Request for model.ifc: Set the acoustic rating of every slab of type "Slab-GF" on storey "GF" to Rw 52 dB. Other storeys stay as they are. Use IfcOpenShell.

First a look at what the model holds.

```python
import ifcopenshell
import ifcopenshell.util.element

model = ifcopenshell.open("model.ifc")
print(model.schema)
storey = next(s for s in model.by_type("IfcBuildingStorey") if s.Name == "GF")
slabs = [e for e in ifcopenshell.util.element.get_decomposition(storey) if e.is_a("IfcSlab")]
seen = {}
for e in slabs:
    element_type = ifcopenshell.util.element.get_type(e)
    key = (element_type.Name if element_type != e and element_type else None, ifcopenshell.util.element.get_pset(e, "Pset_SlabCommon", "AcousticRating"))
    seen[key] = seen.get(key, 0) + 1
for (name, value), count in sorted(seen.items(), key=str):
    print(count, "x", name, "|", value)
```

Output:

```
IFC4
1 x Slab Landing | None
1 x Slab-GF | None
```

```python
import ifcopenshell
import ifcopenshell.api.pset
import ifcopenshell.util.element

model = ifcopenshell.open("model.ifc")

storey = next(s for s in model.by_type("IfcBuildingStorey") if s.Name == "GF")
slabs = [e for e in ifcopenshell.util.element.get_decomposition(storey) if e.is_a("IfcSlab")]

count = 0
for e in slabs:
    element_type = ifcopenshell.util.element.get_type(e)
    if element_type in (None, e) or element_type.Name != "Slab-GF":
        continue
    # add_pset returns the element's existing set when there is one.
    pset = ifcopenshell.api.pset.add_pset(model, product=e, name="Pset_SlabCommon")
    ifcopenshell.api.pset.edit_pset(model, pset=pset, properties={"AcousticRating": "Rw 52 dB"})
    count += 1

print(count, "slabs updated")

model.write("model_updated.ifc")
```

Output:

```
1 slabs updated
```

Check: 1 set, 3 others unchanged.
